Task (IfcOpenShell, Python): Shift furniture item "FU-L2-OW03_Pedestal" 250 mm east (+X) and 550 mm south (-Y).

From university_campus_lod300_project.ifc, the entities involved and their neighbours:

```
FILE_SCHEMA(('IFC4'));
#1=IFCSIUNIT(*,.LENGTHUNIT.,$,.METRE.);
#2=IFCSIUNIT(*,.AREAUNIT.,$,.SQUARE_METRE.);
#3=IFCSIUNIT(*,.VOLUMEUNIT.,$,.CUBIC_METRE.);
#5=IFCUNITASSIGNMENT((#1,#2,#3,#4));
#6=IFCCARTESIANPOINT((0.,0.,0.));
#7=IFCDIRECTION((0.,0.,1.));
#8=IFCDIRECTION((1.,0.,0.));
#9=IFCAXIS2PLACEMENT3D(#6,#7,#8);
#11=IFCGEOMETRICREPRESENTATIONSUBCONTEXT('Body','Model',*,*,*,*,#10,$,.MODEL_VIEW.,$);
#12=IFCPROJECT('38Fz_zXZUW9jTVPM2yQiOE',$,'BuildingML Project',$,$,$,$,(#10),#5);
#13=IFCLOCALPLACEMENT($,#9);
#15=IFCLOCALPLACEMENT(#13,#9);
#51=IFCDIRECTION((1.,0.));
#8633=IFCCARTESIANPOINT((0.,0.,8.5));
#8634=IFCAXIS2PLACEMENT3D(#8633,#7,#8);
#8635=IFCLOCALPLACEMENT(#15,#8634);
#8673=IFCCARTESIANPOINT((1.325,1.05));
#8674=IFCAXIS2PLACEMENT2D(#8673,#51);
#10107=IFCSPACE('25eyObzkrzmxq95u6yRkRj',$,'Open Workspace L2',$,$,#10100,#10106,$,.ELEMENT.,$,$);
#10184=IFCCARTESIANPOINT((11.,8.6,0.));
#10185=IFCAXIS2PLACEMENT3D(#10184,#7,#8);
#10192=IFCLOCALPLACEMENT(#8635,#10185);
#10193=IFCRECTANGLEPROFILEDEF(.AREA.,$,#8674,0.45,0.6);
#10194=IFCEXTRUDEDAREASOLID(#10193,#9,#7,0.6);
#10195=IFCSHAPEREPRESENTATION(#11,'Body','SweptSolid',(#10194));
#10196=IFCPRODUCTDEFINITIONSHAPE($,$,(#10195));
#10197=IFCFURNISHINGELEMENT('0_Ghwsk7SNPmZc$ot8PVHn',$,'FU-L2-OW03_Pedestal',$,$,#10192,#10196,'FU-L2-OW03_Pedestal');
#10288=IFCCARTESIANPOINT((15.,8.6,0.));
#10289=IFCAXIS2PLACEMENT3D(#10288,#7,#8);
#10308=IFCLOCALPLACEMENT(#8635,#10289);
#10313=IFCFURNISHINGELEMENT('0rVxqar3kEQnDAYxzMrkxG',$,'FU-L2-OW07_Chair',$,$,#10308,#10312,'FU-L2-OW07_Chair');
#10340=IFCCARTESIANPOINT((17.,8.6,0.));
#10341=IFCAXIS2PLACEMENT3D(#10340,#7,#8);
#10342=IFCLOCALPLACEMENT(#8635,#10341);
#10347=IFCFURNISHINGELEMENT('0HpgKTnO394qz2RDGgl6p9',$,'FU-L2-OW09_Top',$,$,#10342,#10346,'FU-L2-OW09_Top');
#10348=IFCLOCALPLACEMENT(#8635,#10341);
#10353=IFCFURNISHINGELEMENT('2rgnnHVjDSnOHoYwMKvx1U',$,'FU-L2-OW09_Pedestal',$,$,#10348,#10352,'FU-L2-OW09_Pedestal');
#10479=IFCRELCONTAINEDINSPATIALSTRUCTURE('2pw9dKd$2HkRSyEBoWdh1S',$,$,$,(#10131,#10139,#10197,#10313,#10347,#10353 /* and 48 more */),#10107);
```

```python
import ifcopenshell
import ifcopenshell.api.geometry
import ifcopenshell.util.placement

model = ifcopenshell.open("university_campus_lod300_project.ifc")

item = model.by_id(10197)
matrix = ifcopenshell.util.placement.get_local_placement(item.ObjectPlacement)
matrix[0, 3] += 0.25
matrix[1, 3] -= 0.55
ifcopenshell.api.geometry.edit_object_placement(model, product=item, matrix=matrix, is_si=False)

print(ifcopenshell.util.placement.get_local_placement(item.ObjectPlacement).round(3) + 0.0)

model.write("university_campus_lod300_project_edited.ifc")
```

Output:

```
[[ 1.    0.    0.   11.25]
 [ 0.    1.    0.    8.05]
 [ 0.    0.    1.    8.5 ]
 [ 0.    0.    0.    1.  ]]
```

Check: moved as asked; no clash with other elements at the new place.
